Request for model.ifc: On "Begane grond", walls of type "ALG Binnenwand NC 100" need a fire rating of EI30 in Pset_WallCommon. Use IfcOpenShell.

First a look at what the model holds.

```python
import ifcopenshell
import ifcopenshell.util.element

model = ifcopenshell.open("model.ifc")
print(model.schema)
storey = next(s for s in model.by_type("IfcBuildingStorey") if s.Name == "Begane grond")
walls = [e for e in ifcopenshell.util.element.get_decomposition(storey) if e.is_a("IfcWall")]
seen = {}
for e in walls:
    element_type = ifcopenshell.util.element.get_type(e)
    key = (element_type.Name if element_type != e and element_type else None, ifcopenshell.util.element.get_pset(e, "Pset_WallCommon", "FireRating"))
    seen[key] = seen.get(key, 0) + 1
for (name, value), count in sorted(seen.items(), key=str):
    print(count, "x", name, "|", value)
```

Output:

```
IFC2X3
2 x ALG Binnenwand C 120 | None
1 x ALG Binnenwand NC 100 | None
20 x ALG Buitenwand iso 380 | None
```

```python
import ifcopenshell
import ifcopenshell.api.pset
import ifcopenshell.util.element

model = ifcopenshell.open("model.ifc")

storey = next(s for s in model.by_type("IfcBuildingStorey") if s.Name == "Begane grond")
walls = [e for e in ifcopenshell.util.element.get_decomposition(storey) if e.is_a("IfcWall")]

count = 0
for e in walls:
    element_type = ifcopenshell.util.element.get_type(e)
    if element_type in (None, e) or element_type.Name != "ALG Binnenwand NC 100":
        continue
    # add_pset returns the element's existing set when there is one.
    pset = ifcopenshell.api.pset.add_pset(model, product=e, name="Pset_WallCommon")
    ifcopenshell.api.pset.edit_pset(model, pset=pset, properties={"FireRating": "EI30"})
    count += 1

print(count, "walls updated")

model.write("model_updated.ifc")
```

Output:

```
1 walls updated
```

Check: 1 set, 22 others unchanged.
